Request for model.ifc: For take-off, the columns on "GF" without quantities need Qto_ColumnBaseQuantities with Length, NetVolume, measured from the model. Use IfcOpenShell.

First a look at what the model holds.

```python
import ifcopenshell
import ifcopenshell.util.element
import ifcopenshell.util.unit

model = ifcopenshell.open("model.ifc")
print(model.schema)
for unit_type in ("LENGTHUNIT", "AREAUNIT", "VOLUMEUNIT"):
    print(unit_type, ifcopenshell.util.unit.calculate_unit_scale(model, unit_type))
storey = next(s for s in model.by_type("IfcBuildingStorey") if s.Name == "GF")
columns = [e for e in ifcopenshell.util.element.get_decomposition(storey) if e.is_a("IfcColumn")]
for e in sorted(columns, key=lambda e: e.id()):
    print(e.id(), e.is_a(), e.Name, list(ifcopenshell.util.element.get_psets(e, qtos_only=True)), sep=" | ")
```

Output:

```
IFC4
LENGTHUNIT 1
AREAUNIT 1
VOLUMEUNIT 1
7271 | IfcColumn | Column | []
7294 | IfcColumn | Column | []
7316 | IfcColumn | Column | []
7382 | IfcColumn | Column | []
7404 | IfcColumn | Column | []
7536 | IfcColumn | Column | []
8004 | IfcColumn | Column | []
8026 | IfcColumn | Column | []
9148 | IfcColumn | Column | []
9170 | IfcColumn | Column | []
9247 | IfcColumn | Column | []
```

```python
import ifcopenshell
import ifcopenshell.api.pset
import ifcopenshell.geom
import ifcopenshell.util.element
import ifcopenshell.util.shape
import ifcopenshell.util.unit

model = ifcopenshell.open("model.ifc")
unit_scale = ifcopenshell.util.unit.calculate_unit_scale(model)
volume_scale = ifcopenshell.util.unit.calculate_unit_scale(model, "VOLUMEUNIT")
settings = ifcopenshell.geom.settings()

storey = next(s for s in model.by_type("IfcBuildingStorey") if s.Name == "GF")
columns = [e for e in ifcopenshell.util.element.get_decomposition(storey) if e.is_a("IfcColumn")]

for e in sorted(columns, key=lambda e: e.id()):
    if ifcopenshell.util.element.get_psets(e, qtos_only=True, should_inherit=False):
        continue
    # Geometry comes back in metres, in the element's own axes.
    shape = ifcopenshell.geom.create_shape(settings, e)
    values = {
        "Length": ifcopenshell.util.shape.get_z(shape.geometry) / unit_scale,
        "NetVolume": ifcopenshell.util.shape.get_volume(shape.geometry) / volume_scale,
    }
    qto = ifcopenshell.api.pset.add_qto(model, product=e, name="Qto_ColumnBaseQuantities")
    ifcopenshell.api.pset.edit_qto(model, qto=qto, properties=values)
    print(e.id(), {k: round(v, 3) for k, v in values.items()})

model.write("model_rev.ifc")
```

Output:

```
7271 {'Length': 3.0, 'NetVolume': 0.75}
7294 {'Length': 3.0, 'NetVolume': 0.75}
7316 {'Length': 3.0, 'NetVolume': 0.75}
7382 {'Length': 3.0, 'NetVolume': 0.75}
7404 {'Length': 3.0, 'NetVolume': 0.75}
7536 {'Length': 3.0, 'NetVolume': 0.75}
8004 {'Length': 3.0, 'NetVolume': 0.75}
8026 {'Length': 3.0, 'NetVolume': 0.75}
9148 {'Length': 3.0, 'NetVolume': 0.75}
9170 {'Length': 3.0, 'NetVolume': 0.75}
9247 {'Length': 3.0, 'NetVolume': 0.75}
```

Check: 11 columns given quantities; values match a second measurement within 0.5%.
